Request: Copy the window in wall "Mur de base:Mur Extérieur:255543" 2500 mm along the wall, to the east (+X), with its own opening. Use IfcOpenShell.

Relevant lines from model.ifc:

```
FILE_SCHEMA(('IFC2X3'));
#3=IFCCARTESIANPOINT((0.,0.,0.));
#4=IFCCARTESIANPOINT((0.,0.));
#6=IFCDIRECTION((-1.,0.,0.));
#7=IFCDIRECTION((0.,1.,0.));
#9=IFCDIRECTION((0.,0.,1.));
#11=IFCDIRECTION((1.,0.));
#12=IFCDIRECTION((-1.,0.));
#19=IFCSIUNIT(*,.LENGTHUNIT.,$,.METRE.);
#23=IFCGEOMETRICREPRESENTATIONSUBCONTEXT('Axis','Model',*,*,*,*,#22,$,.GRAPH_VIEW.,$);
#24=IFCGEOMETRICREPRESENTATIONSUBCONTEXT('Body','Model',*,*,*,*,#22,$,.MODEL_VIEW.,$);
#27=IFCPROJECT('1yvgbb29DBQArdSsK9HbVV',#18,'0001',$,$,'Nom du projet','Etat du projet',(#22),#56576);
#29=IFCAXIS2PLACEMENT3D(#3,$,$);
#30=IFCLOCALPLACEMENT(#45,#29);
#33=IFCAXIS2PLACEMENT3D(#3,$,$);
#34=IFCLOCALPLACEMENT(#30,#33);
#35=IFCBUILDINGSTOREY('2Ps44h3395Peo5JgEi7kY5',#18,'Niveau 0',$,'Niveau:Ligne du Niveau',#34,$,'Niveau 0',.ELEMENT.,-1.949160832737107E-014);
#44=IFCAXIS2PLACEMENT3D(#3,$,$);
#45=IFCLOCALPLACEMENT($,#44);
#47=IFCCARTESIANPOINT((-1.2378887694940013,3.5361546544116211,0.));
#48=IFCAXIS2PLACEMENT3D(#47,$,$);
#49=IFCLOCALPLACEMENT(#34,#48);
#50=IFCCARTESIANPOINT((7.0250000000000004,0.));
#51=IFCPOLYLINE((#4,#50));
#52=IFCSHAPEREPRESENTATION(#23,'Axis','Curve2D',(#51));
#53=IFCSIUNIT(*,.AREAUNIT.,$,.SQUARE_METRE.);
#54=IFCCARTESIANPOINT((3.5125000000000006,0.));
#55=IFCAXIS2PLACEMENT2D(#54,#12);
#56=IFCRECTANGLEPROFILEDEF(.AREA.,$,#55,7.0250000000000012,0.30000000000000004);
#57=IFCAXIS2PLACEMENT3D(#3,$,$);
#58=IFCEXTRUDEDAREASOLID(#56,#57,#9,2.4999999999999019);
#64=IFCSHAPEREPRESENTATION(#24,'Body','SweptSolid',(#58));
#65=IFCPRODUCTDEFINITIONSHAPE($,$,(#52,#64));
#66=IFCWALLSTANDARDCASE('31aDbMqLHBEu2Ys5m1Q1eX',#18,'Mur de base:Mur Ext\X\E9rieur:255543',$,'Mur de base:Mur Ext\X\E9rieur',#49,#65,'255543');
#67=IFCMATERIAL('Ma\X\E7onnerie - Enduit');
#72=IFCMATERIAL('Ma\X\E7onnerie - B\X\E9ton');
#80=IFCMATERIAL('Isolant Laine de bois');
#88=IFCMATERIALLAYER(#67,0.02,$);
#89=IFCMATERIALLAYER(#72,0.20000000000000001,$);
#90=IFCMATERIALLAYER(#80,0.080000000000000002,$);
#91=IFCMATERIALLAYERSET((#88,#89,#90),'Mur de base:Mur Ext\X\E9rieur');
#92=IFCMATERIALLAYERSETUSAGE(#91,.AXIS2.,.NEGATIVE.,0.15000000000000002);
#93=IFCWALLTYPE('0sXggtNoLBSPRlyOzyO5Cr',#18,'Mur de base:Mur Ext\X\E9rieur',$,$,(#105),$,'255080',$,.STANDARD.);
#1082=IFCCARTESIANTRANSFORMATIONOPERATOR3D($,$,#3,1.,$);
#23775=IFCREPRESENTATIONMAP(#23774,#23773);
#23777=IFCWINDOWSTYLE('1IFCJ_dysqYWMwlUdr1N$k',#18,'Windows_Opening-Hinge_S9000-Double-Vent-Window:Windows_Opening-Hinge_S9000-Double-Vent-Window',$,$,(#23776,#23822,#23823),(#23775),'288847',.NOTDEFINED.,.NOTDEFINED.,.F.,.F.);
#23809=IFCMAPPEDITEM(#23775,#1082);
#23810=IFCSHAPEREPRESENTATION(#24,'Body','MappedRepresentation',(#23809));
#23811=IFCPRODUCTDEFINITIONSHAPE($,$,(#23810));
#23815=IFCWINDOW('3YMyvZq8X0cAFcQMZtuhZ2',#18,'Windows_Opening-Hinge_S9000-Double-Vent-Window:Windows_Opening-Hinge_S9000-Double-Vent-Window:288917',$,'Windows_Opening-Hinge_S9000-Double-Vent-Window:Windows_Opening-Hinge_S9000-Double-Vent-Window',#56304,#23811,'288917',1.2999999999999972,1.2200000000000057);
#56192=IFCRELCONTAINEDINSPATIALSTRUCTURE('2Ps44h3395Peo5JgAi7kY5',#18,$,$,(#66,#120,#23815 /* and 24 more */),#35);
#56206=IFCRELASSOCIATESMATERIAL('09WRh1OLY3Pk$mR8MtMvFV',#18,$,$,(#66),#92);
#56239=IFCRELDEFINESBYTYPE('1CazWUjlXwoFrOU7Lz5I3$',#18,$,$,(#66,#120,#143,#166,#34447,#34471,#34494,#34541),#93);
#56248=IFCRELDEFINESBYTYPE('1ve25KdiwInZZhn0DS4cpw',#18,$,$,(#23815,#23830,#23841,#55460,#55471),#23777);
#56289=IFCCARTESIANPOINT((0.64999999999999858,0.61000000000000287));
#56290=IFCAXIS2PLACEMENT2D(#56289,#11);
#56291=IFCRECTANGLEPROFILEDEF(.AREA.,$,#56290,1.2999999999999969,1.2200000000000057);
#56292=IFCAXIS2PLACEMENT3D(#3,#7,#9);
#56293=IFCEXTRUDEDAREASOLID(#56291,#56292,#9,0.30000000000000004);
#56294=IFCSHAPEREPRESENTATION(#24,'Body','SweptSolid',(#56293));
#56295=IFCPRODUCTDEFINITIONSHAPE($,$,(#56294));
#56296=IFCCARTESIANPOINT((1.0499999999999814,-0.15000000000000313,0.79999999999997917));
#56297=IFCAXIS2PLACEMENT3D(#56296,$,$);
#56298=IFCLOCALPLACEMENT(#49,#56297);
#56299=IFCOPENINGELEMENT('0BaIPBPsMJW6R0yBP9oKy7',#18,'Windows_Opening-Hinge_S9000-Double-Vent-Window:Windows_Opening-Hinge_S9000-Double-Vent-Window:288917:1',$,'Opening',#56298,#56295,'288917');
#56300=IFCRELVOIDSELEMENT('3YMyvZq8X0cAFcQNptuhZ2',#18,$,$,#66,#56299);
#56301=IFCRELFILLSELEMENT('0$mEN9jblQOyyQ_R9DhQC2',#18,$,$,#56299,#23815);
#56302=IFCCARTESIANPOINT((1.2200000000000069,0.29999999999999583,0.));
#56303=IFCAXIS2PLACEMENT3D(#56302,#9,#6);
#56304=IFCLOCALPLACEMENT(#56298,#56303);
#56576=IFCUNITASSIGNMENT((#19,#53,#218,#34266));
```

```python
import ifcopenshell
import ifcopenshell.api.feature
import ifcopenshell.api.geometry
import ifcopenshell.api.root
import ifcopenshell.geom
import ifcopenshell.util.element
import ifcopenshell.util.placement
import ifcopenshell.util.shape
import ifcopenshell.util.unit

model = ifcopenshell.open("model.ifc")
unit_scale = ifcopenshell.util.unit.calculate_unit_scale(model)
settings = ifcopenshell.geom.settings()


def volume(element):
    """Net volume in cubic metres, openings subtracted."""
    shape = ifcopenshell.geom.create_shape(settings, element)
    return ifcopenshell.util.shape.get_volume(shape.geometry)


def reuse_history(source, copy):
    """copy_class also copies each property set's owner history, people and application; keep the originals."""
    for rel in copy.IsDefinedBy:
        if rel.is_a("IfcRelDefinesByProperties") and (history := rel.RelatingPropertyDefinition.OwnerHistory):
            rel.RelatingPropertyDefinition.OwnerHistory = source.OwnerHistory
            ifcopenshell.util.element.remove_deep2(model, history)


window = model.by_guid("3YMyvZq8X0cAFcQMZtuhZ2")
opening = window.FillsVoids[0].RelatingOpeningElement
wall = opening.VoidsElements[0].RelatingBuildingElement
before = volume(wall)
shift = ifcopenshell.util.placement.get_local_placement(wall.ObjectPlacement)[:3, 0] * 2.5 / unit_scale

# copy_class copies the void relationship, type, container and properties, but no geometry.
new_opening = ifcopenshell.api.root.copy_class(model, product=opening)
new_opening.Representation = ifcopenshell.util.element.copy_deep(
    model, opening.Representation, exclude=["IfcGeometricRepresentationContext", "IfcRepresentationMap"]
)
new_opening.Name = "Windows_Opening-Hinge_S9000-Double-Vent-Window:Windows_Opening-Hinge_S9000-Double-Vent-Window"
new_opening.Tag = None
new_window = ifcopenshell.api.root.copy_class(model, product=window)
new_window.Representation = ifcopenshell.util.element.copy_deep(
    model, window.Representation, exclude=["IfcGeometricRepresentationContext", "IfcRepresentationMap"]
)
new_window.Name = "Windows_Opening-Hinge_S9000-Double-Vent-Window:Windows_Opening-Hinge_S9000-Double-Vent-Window"
new_window.Tag = None
reuse_history(window, new_window)
fills = ifcopenshell.api.feature.add_filling(model, opening=new_opening, element=new_window)
fills.OwnerHistory = new_window.OwnerHistory  # required in IFC2X3

for old, new in ((opening, new_opening), (window, new_window)):
    matrix = ifcopenshell.util.placement.get_local_placement(old.ObjectPlacement)
    matrix[:3, 3] += shift
    ifcopenshell.api.geometry.edit_object_placement(model, product=new, matrix=matrix, is_si=False)

after = volume(wall)

print(f"wall volume {before:.3f} -> {after:.3f} m3")

model.write("model_rev.ifc")
```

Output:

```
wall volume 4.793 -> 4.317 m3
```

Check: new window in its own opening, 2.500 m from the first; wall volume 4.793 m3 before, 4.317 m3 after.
